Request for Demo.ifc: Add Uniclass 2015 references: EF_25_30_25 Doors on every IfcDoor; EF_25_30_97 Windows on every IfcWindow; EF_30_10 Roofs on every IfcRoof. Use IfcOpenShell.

First a look at what the model holds.

```python
import ifcopenshell

model = ifcopenshell.open("Demo.ifc")
print(model.schema)
print("classifications:", [c.Name for c in model.by_type("IfcClassification")])
for ifc_class in ("IfcDoor", "IfcRoof", "IfcStair", "IfcWall", "IfcWindow"):
    print(ifc_class, len(model.by_type(ifc_class)))
```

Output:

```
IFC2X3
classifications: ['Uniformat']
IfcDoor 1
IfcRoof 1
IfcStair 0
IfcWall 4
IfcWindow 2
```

```python
import ifcopenshell
import ifcopenshell.api.classification

model = ifcopenshell.open("Demo.ifc")

# IFC2X3 requires Source and Edition and has no link from the project to the system.
system = model.create_entity("IfcClassification", Source="NBS", Edition="2015", Name="Uniclass 2015")

codes = {
    "IfcDoor": ("EF_25_30_25", "Doors"),
    "IfcWindow": ("EF_25_30_97", "Windows"),
    "IfcRoof": ("EF_30_10", "Roofs"),
}
for ifc_class, (code, name) in codes.items():
    products = model.by_type(ifc_class)
    ifcopenshell.api.classification.add_reference(
        model, products=products, classification=system, identification=code, name=name
    )
    print(code, len(products))

model.write("Demo_v2.ifc")
```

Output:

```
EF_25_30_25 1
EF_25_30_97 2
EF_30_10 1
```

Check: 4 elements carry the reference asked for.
